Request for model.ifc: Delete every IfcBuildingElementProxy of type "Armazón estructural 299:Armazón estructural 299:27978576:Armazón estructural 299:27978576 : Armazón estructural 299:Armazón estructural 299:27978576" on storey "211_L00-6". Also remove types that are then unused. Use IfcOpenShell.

First a look at what the model holds.

```python
import ifcopenshell
import ifcopenshell.util.element

model = ifcopenshell.open("model.ifc")
print(model.schema)
storey = next(s for s in model.by_type("IfcBuildingStorey") if s.Name == "211_L00-6")
proxies = [e for e in ifcopenshell.util.element.get_decomposition(storey) if e.is_a("IfcBuildingElementProxy")]
seen = {}
for e in proxies:
    element_type = ifcopenshell.util.element.get_type(e)
    name = element_type.Name if element_type not in (None, e) else None
    seen[name] = seen.get(name, 0) + 1
for name, count in sorted(seen.items(), key=str):
    print(count, "x", name)
```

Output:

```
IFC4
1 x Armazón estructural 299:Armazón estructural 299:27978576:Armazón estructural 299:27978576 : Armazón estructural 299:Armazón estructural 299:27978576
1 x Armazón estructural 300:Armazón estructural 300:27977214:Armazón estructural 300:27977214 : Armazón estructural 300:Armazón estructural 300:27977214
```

```python
import ifcopenshell
import ifcopenshell.api.root
import ifcopenshell.util.element

model = ifcopenshell.open("model.ifc")

storey = next(s for s in model.by_type("IfcBuildingStorey") if s.Name == "211_L00-6")
proxies = [e for e in ifcopenshell.util.element.get_decomposition(storey) if e.is_a("IfcBuildingElementProxy")]
targets = [e for e in proxies if (t := ifcopenshell.util.element.get_type(e)) not in (None, e) and t.Name == "Armazón estructural 299:Armazón estructural 299:27978576:Armazón estructural 299:27978576 : Armazón estructural 299:Armazón estructural 299:27978576"]
types = {ifcopenshell.util.element.get_type(e) for e in targets} - {None, *targets}

for e in targets:
    ifcopenshell.api.root.remove_product(model, product=e)
print(len(targets), "removed")

unused = [t for t in types if not ifcopenshell.util.element.get_types(t)]
for t in unused:
    ifcopenshell.api.root.remove_product(model, product=t)
print(len(unused), "unused types removed")

model.write("model_edited.ifc")
```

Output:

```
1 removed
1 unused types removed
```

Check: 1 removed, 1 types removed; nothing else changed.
